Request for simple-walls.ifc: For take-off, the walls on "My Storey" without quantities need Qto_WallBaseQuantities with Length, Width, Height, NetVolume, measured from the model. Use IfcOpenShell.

First a look at what the model holds.

```python
import ifcopenshell
import ifcopenshell.util.element
import ifcopenshell.util.unit

model = ifcopenshell.open("simple-walls.ifc")
print(model.schema)
for unit_type in ("LENGTHUNIT", "AREAUNIT", "VOLUMEUNIT"):
    print(unit_type, ifcopenshell.util.unit.calculate_unit_scale(model, unit_type))
storey = next(s for s in model.by_type("IfcBuildingStorey") if s.Name == "My Storey")
walls = [e for e in ifcopenshell.util.element.get_decomposition(storey) if e.is_a("IfcWall")]
for e in sorted(walls, key=lambda e: e.id()):
    print(e.id(), e.is_a(), e.Name, list(ifcopenshell.util.element.get_psets(e, qtos_only=True)), sep=" | ")
```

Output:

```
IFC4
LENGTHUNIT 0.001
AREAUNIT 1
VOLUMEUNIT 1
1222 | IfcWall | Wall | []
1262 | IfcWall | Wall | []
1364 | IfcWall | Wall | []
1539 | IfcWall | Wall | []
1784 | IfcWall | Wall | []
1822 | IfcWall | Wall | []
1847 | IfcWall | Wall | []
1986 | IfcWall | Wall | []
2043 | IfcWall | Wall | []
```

```python
import ifcopenshell
import ifcopenshell.api.pset
import ifcopenshell.geom
import ifcopenshell.util.element
import ifcopenshell.util.shape
import ifcopenshell.util.unit

model = ifcopenshell.open("simple-walls.ifc")
unit_scale = ifcopenshell.util.unit.calculate_unit_scale(model)
volume_scale = ifcopenshell.util.unit.calculate_unit_scale(model, "VOLUMEUNIT")
settings = ifcopenshell.geom.settings()

storey = next(s for s in model.by_type("IfcBuildingStorey") if s.Name == "My Storey")
walls = [e for e in ifcopenshell.util.element.get_decomposition(storey) if e.is_a("IfcWall")]

for e in sorted(walls, key=lambda e: e.id()):
    if ifcopenshell.util.element.get_psets(e, qtos_only=True, should_inherit=False):
        continue
    # Geometry comes back in metres, in the element's own axes.
    shape = ifcopenshell.geom.create_shape(settings, e)
    values = {
        "Length": ifcopenshell.util.shape.get_x(shape.geometry) / unit_scale,
        "Width": ifcopenshell.util.shape.get_y(shape.geometry) / unit_scale,
        "Height": ifcopenshell.util.shape.get_z(shape.geometry) / unit_scale,
        "NetVolume": ifcopenshell.util.shape.get_volume(shape.geometry) / volume_scale,
    }
    qto = ifcopenshell.api.pset.add_qto(model, product=e, name="Qto_WallBaseQuantities")
    ifcopenshell.api.pset.edit_qto(model, qto=qto, properties=values)
    print(e.id(), {k: round(v, 3) for k, v in values.items()})

model.write("simple-walls-out.ifc")
```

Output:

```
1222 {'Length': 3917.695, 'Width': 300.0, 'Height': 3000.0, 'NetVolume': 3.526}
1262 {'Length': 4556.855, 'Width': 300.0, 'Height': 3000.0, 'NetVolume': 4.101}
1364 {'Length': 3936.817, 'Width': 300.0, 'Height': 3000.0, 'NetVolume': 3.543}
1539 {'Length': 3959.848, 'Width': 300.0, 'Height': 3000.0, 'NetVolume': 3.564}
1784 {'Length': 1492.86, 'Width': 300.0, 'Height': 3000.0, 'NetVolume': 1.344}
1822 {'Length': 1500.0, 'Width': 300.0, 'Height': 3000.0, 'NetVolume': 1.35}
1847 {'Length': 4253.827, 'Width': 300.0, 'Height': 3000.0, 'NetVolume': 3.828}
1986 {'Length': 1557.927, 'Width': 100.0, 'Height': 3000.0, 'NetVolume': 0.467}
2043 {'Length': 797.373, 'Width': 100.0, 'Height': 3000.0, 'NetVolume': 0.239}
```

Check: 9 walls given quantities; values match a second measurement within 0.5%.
